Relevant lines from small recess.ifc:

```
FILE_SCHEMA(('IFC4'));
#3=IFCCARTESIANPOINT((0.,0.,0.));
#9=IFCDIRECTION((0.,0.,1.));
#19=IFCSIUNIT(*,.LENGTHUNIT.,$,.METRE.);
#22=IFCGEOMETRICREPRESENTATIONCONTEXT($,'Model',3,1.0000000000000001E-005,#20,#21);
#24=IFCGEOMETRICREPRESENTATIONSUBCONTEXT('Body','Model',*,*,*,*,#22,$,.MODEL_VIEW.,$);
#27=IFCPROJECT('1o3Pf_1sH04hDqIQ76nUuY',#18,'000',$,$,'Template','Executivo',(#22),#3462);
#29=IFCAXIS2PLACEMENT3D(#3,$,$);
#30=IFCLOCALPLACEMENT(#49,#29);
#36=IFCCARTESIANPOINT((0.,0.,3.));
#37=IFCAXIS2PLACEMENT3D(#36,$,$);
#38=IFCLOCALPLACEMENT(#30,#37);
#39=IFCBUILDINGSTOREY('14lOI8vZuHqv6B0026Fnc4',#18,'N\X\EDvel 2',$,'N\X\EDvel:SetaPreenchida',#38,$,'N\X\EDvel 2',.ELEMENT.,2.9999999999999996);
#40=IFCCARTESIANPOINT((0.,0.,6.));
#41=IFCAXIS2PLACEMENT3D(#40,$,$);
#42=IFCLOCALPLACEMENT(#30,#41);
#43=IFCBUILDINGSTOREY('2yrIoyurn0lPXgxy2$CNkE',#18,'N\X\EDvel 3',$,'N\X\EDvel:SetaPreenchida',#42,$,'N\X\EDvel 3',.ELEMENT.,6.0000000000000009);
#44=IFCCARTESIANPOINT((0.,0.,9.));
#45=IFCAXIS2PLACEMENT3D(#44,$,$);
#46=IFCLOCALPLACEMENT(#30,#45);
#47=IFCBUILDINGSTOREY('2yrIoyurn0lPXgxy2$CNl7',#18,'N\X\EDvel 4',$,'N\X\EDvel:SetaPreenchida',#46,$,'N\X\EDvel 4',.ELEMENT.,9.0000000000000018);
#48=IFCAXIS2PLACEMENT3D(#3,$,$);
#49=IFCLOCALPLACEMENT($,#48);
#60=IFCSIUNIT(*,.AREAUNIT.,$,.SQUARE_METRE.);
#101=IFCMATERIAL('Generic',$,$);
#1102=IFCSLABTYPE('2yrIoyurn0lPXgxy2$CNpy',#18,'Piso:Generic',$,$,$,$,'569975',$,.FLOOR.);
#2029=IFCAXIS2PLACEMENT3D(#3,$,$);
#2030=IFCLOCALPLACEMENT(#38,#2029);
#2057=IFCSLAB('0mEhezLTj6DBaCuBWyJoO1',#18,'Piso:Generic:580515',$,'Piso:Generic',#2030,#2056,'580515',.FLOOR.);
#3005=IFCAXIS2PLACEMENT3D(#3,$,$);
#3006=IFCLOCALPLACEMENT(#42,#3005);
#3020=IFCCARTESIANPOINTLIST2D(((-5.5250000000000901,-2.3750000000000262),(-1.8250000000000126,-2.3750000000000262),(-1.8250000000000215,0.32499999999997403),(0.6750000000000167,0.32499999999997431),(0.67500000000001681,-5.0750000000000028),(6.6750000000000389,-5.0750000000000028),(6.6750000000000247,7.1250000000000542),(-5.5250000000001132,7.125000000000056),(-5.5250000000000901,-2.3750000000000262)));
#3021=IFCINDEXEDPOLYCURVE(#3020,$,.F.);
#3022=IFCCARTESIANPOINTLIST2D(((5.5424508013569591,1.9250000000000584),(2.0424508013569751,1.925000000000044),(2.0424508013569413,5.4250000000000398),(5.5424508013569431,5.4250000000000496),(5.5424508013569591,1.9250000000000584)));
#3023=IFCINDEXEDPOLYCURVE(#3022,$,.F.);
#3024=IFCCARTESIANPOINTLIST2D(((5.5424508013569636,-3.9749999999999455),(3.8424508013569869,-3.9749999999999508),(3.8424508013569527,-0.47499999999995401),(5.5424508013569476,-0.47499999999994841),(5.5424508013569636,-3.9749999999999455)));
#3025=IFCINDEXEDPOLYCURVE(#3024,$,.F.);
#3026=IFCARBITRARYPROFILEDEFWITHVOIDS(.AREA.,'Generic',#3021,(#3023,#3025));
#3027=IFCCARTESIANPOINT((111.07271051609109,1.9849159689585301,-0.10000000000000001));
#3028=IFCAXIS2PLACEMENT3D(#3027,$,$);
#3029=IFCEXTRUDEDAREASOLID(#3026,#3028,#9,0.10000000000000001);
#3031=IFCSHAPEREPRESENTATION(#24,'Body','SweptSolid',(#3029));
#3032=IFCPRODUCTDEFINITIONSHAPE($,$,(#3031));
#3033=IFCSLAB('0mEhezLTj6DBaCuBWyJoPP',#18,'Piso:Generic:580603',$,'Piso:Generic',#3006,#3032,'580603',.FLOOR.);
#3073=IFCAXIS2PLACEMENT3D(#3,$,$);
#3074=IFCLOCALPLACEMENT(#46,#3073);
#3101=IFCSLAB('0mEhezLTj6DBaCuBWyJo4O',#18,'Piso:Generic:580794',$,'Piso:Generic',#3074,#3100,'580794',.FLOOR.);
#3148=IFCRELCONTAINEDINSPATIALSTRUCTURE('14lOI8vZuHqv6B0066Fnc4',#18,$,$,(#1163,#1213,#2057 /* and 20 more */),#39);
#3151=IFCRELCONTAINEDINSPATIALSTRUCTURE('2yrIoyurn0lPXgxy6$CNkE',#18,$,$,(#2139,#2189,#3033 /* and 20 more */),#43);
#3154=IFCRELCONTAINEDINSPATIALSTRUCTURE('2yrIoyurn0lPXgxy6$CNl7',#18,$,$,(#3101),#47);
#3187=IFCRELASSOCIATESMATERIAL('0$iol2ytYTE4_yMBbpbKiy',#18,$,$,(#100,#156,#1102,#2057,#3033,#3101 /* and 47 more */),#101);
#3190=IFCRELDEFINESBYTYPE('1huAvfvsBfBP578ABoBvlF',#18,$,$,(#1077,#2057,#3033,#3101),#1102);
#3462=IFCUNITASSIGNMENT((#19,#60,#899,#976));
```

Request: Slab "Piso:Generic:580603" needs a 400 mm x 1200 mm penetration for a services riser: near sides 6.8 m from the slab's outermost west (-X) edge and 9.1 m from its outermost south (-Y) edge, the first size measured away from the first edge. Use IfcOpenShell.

```python
import numpy as np
import ifcopenshell
import ifcopenshell.api.feature
import ifcopenshell.api.geometry
import ifcopenshell.api.root
import ifcopenshell.geom
import ifcopenshell.util.placement
import ifcopenshell.util.representation
import ifcopenshell.util.shape
import ifcopenshell.util.unit

model = ifcopenshell.open("small recess.ifc")
unit_scale = ifcopenshell.util.unit.calculate_unit_scale(model)
settings = ifcopenshell.geom.settings()


def volume(element):
    """Net volume in cubic metres, openings subtracted."""
    shape = ifcopenshell.geom.create_shape(settings, element)
    return ifcopenshell.util.shape.get_volume(shape.geometry)


slab = model.by_guid("0mEhezLTj6DBaCuBWyJoPP")
before = volume(slab)

# Extent in the slab's own axes, in metres. The edges named are its -X and -Y sides.
slab_shape = ifcopenshell.geom.create_shape(settings, slab)
vertices = ifcopenshell.util.shape.get_vertices(slab_shape.geometry)
x_min, y_min, bottom = vertices.min(axis=0)
top = vertices[:, 2].max()

opening = ifcopenshell.api.root.create_entity(model, ifc_class="IfcOpeningElement", name="Services riser opening", predefined_type="OPENING")
context = ifcopenshell.util.representation.get_context(model, "Model", "Body", "MODEL_VIEW")
width, depth = 0.4, 1.2
outline = [(0.0, 0.0), (width, 0.0), (width, depth), (0.0, depth), (0.0, 0.0)]
# Overshoot both faces by 50 mm so the cut is clean.
shape = ifcopenshell.api.geometry.add_slab_representation(
    model, context=context, depth=top - bottom + 0.1, polyline=outline
)
ifcopenshell.api.geometry.assign_representation(model, product=opening, representation=shape)

matrix = ifcopenshell.util.placement.get_local_placement(slab.ObjectPlacement)
matrix[:, 3] = matrix @ np.append(np.array([x_min + 6.8, y_min + 9.1, bottom - 0.05]) / unit_scale, 1.0)
ifcopenshell.api.geometry.edit_object_placement(model, product=opening, matrix=matrix, is_si=False)
ifcopenshell.api.feature.add_feature(model, feature=opening, element=slab)

after = volume(slab)

print(f"slab volume {before:.3f} -> {after:.3f} m3")

model.write("small recess_rev.ifc")
```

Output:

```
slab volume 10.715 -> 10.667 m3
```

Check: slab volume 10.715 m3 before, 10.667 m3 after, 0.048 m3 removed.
